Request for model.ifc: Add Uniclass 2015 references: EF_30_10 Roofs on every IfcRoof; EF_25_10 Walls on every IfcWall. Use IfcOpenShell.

First a look at what the model holds.

```python
import ifcopenshell

model = ifcopenshell.open("model.ifc")
print(model.schema)
print("classifications:", [c.Name for c in model.by_type("IfcClassification")])
for ifc_class in ("IfcDoor", "IfcRoof", "IfcStair", "IfcWall", "IfcWindow"):
    print(ifc_class, len(model.by_type(ifc_class)))
```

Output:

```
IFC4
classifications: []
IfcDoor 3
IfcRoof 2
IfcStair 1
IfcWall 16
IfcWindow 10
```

```python
import ifcopenshell
import ifcopenshell.api.classification

model = ifcopenshell.open("model.ifc")

system = ifcopenshell.api.classification.add_classification(model, classification="Uniclass 2015")

codes = {
    "IfcRoof": ("EF_30_10", "Roofs"),
    "IfcWall": ("EF_25_10", "Walls"),
}
for ifc_class, (code, name) in codes.items():
    products = model.by_type(ifc_class)
    ifcopenshell.api.classification.add_reference(
        model, products=products, classification=system, identification=code, name=name
    )
    print(code, len(products))

model.write("model_rev.ifc")
```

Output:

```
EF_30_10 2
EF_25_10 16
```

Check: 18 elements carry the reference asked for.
